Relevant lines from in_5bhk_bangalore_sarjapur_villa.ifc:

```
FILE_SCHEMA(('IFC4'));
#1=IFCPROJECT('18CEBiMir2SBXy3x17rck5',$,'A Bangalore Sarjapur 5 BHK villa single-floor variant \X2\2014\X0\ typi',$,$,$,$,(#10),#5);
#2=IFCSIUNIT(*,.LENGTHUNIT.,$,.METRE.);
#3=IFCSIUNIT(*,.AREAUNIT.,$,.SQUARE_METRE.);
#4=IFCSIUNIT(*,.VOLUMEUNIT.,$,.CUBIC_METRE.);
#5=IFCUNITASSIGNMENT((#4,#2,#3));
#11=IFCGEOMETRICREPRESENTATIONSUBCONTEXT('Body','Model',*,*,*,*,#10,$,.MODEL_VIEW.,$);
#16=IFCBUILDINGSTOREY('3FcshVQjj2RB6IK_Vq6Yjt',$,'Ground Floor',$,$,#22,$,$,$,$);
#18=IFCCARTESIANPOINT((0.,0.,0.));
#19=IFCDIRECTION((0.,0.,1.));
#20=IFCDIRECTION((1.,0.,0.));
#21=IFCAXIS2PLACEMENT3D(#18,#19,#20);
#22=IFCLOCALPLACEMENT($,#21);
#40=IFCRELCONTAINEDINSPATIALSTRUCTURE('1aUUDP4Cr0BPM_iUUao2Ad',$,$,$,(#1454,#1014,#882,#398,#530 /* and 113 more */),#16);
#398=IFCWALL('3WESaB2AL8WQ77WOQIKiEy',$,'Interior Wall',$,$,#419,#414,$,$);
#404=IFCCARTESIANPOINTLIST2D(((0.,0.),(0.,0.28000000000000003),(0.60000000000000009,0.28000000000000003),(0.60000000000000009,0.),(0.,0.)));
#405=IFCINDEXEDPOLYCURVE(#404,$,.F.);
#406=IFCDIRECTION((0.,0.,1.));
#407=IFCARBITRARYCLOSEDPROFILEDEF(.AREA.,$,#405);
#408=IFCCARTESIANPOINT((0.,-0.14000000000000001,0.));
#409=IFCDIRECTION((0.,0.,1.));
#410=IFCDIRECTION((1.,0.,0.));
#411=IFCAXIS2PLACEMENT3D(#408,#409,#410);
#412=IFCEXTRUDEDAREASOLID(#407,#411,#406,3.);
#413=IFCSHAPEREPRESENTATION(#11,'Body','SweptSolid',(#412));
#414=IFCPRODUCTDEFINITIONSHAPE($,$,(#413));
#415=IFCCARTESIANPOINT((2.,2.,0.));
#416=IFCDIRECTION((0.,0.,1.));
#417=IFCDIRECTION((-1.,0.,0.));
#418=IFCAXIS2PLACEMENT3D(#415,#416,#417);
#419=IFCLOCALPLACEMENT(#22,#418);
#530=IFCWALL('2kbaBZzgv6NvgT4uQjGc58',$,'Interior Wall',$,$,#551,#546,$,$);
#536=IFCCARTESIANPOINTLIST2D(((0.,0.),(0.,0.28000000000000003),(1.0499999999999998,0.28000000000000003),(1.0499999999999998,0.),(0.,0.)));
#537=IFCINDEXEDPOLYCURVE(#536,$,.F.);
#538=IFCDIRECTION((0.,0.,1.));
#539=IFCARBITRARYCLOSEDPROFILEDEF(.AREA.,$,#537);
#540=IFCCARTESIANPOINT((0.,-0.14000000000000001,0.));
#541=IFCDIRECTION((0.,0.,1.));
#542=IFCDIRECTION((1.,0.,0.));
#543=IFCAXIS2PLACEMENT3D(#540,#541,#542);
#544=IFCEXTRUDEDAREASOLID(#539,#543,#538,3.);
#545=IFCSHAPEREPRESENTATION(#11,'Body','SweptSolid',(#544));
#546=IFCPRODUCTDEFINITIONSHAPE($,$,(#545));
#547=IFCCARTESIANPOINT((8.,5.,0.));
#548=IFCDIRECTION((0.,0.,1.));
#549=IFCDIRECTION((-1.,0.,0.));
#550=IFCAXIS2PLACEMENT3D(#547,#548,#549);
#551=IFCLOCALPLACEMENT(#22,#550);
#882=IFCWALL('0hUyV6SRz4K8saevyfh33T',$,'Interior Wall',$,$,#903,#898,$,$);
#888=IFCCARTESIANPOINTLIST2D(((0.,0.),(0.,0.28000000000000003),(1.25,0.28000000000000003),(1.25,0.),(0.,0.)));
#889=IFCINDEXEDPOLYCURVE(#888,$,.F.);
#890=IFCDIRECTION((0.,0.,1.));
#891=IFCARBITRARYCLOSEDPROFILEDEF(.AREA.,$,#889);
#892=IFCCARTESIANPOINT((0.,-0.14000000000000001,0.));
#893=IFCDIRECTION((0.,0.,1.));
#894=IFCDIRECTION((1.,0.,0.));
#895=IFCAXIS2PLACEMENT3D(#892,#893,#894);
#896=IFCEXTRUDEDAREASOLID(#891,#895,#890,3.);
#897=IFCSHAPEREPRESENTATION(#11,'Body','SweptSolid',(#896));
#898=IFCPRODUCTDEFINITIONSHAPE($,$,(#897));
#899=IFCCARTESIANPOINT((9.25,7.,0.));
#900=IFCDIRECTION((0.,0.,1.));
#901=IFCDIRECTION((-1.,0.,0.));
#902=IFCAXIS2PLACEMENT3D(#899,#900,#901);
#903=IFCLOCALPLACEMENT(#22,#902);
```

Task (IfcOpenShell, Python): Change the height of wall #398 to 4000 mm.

```python
import ifcopenshell
import ifcopenshell.geom
import ifcopenshell.util.representation
import ifcopenshell.util.shape
import ifcopenshell.util.unit

model = ifcopenshell.open("in_5bhk_bangalore_sarjapur_villa.ifc")
unit_scale = ifcopenshell.util.unit.calculate_unit_scale(model)
settings = ifcopenshell.geom.settings()


def volume(element):
    """Net volume in cubic metres, openings subtracted."""
    shape = ifcopenshell.geom.create_shape(settings, element)
    return ifcopenshell.util.shape.get_volume(shape.geometry)


wall = model.by_guid("3WESaB2AL8WQ77WOQIKiEy")
before = volume(wall)

body = ifcopenshell.util.representation.get_representation(wall, "Model", "Body")
solid = body.Items[0]
old_height = solid.Depth
solid.Depth = 4 / unit_scale
after = volume(wall)

print(f"height {old_height:g} -> {solid.Depth:g}, volume {before:.3f} -> {after:.3f} m3")

model.write("in_5bhk_bangalore_sarjapur_villa_rev.ifc")
```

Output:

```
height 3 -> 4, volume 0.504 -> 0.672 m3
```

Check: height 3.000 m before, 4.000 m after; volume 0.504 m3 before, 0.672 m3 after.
